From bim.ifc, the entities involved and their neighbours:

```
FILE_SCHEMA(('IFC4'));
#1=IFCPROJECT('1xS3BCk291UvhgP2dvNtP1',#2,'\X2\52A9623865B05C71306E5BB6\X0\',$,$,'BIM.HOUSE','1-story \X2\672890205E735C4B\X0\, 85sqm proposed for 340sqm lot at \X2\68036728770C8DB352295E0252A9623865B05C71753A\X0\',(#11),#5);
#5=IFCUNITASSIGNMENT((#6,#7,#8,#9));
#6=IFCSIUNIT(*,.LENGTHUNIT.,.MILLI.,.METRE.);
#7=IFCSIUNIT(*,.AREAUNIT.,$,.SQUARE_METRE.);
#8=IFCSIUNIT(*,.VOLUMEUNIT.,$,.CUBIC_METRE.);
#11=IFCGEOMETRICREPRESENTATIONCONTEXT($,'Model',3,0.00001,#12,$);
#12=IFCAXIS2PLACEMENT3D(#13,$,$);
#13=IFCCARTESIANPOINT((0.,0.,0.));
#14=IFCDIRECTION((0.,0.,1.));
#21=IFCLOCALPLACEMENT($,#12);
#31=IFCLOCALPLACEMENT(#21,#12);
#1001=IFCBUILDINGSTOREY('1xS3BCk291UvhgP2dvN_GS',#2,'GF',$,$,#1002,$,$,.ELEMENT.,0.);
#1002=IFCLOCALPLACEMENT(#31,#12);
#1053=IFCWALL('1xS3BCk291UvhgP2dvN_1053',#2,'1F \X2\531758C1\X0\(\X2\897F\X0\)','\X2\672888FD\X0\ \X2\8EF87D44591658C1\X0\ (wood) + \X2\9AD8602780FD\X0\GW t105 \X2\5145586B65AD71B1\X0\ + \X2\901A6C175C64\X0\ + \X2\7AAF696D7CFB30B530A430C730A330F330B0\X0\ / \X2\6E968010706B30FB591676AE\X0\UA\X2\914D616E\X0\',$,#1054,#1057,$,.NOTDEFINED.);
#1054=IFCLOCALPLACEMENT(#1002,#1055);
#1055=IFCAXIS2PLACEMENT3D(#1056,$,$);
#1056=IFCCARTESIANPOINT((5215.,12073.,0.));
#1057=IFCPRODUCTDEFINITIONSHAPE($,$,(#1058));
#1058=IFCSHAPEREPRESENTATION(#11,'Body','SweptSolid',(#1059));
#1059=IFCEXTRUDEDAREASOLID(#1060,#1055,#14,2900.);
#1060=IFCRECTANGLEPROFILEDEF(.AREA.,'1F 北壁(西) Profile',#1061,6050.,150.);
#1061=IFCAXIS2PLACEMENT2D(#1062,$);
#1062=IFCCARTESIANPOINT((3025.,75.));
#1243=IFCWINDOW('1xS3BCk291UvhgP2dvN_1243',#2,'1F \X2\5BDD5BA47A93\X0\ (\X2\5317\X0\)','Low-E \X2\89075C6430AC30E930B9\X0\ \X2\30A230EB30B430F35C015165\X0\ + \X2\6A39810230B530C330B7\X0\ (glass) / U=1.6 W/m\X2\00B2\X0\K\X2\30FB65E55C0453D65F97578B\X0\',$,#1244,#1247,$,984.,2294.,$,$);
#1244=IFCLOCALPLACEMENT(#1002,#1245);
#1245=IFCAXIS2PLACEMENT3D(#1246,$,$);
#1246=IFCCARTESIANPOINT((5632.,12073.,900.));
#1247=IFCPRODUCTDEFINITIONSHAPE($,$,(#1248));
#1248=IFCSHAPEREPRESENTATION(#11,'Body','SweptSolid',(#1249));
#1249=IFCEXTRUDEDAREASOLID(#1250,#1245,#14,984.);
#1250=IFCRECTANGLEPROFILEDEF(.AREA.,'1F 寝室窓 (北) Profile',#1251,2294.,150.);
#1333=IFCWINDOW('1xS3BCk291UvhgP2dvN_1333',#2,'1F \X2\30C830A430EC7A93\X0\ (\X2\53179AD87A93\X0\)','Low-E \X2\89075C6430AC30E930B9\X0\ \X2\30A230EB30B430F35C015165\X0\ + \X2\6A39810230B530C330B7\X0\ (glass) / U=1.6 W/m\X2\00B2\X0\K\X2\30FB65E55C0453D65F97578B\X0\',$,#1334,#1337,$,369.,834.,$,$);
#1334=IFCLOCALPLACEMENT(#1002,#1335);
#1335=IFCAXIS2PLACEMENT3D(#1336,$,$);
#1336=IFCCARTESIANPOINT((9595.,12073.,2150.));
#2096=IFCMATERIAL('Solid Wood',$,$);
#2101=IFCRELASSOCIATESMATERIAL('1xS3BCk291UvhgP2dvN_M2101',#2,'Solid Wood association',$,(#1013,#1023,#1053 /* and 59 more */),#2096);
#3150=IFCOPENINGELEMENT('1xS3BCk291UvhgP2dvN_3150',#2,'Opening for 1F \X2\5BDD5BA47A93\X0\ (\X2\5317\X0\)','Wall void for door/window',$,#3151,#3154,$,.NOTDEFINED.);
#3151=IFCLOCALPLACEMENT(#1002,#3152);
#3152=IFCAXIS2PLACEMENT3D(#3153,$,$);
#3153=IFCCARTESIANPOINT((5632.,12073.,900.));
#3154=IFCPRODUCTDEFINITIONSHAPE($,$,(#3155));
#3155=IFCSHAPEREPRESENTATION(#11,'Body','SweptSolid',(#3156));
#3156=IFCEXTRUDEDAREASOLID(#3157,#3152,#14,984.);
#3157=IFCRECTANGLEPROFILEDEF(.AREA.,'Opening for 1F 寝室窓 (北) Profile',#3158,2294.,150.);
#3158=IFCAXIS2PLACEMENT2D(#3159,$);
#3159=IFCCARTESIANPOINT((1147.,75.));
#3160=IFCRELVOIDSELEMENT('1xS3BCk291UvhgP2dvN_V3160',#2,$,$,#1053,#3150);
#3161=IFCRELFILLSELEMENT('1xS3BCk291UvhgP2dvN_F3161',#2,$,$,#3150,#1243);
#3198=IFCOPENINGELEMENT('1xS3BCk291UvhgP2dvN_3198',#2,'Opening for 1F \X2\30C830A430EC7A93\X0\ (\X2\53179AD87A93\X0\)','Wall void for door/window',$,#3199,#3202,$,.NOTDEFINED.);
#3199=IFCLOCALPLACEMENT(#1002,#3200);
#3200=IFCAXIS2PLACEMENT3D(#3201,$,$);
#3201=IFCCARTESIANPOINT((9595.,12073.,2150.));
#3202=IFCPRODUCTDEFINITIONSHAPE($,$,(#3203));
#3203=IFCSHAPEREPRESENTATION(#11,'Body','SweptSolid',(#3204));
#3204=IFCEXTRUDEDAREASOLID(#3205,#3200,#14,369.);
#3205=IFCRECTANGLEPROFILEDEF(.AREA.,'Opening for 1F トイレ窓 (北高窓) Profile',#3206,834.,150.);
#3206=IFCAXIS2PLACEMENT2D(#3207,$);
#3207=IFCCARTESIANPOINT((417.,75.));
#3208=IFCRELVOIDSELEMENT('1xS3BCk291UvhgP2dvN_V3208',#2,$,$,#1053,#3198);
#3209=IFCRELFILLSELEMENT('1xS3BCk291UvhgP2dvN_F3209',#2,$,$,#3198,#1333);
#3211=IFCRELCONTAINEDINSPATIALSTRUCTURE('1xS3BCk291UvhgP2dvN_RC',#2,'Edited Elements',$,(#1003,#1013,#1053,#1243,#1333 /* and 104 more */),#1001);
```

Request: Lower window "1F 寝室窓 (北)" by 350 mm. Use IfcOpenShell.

```python
import numpy as np
import ifcopenshell
import ifcopenshell.api.geometry
import ifcopenshell.util.placement
import ifcopenshell.util.unit

model = ifcopenshell.open("bim.ifc")
unit_scale = ifcopenshell.util.unit.calculate_unit_scale(model)

window = model.by_id(1243)
opening = window.FillsVoids[0].RelatingOpeningElement
dz = -0.35 / unit_scale

shift = np.array([0.0, 0.0, dz])
# The window is not placed relative to its opening, so move both.
for product in (opening, window):
    matrix = ifcopenshell.util.placement.get_local_placement(product.ObjectPlacement)
    matrix[:3, 3] += shift
    ifcopenshell.api.geometry.edit_object_placement(model, product=product, matrix=matrix, is_si=False)

print(f"moved by {dz * unit_scale:+.3f} m")

model.write("bim_edited.ifc")
```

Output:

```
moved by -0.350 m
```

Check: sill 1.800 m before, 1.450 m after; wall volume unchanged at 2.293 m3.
